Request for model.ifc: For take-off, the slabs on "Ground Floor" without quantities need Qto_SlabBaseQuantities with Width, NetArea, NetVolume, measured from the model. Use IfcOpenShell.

First a look at what the model holds.

```python
import ifcopenshell
import ifcopenshell.util.element
import ifcopenshell.util.unit

model = ifcopenshell.open("model.ifc")
print(model.schema)
for unit_type in ("LENGTHUNIT", "AREAUNIT", "VOLUMEUNIT"):
    print(unit_type, ifcopenshell.util.unit.calculate_unit_scale(model, unit_type))
storey = next(s for s in model.by_type("IfcBuildingStorey") if s.Name == "Ground Floor")
slabs = [e for e in ifcopenshell.util.element.get_decomposition(storey) if e.is_a("IfcSlab")]
for e in sorted(slabs, key=lambda e: e.id()):
    print(e.id(), e.is_a(), e.Name, list(ifcopenshell.util.element.get_psets(e, qtos_only=True)), sep=" | ")
```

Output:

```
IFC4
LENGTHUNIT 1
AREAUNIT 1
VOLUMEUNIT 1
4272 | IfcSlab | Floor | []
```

```python
import ifcopenshell
import ifcopenshell.api.pset
import ifcopenshell.geom
import ifcopenshell.util.element
import ifcopenshell.util.shape
import ifcopenshell.util.unit

model = ifcopenshell.open("model.ifc")
unit_scale = ifcopenshell.util.unit.calculate_unit_scale(model)
area_scale = ifcopenshell.util.unit.calculate_unit_scale(model, "AREAUNIT")
volume_scale = ifcopenshell.util.unit.calculate_unit_scale(model, "VOLUMEUNIT")
settings = ifcopenshell.geom.settings()

storey = next(s for s in model.by_type("IfcBuildingStorey") if s.Name == "Ground Floor")
slabs = [e for e in ifcopenshell.util.element.get_decomposition(storey) if e.is_a("IfcSlab")]

for e in sorted(slabs, key=lambda e: e.id()):
    if ifcopenshell.util.element.get_psets(e, qtos_only=True, should_inherit=False):
        continue
    # Geometry comes back in metres, in the element's own axes.
    shape = ifcopenshell.geom.create_shape(settings, e)
    values = {
        "Width": ifcopenshell.util.shape.get_z(shape.geometry) / unit_scale,
        "NetArea": ifcopenshell.util.shape.get_footprint_area(shape.geometry) / area_scale,
        "NetVolume": ifcopenshell.util.shape.get_volume(shape.geometry) / volume_scale,
    }
    qto = ifcopenshell.api.pset.add_qto(model, product=e, name="Qto_SlabBaseQuantities")
    ifcopenshell.api.pset.edit_qto(model, qto=qto, properties=values)
    print(e.id(), {k: round(v, 3) for k, v in values.items()})

model.write("model-out.ifc")
```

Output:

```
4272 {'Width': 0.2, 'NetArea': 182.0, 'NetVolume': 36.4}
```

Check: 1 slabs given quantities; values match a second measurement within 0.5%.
